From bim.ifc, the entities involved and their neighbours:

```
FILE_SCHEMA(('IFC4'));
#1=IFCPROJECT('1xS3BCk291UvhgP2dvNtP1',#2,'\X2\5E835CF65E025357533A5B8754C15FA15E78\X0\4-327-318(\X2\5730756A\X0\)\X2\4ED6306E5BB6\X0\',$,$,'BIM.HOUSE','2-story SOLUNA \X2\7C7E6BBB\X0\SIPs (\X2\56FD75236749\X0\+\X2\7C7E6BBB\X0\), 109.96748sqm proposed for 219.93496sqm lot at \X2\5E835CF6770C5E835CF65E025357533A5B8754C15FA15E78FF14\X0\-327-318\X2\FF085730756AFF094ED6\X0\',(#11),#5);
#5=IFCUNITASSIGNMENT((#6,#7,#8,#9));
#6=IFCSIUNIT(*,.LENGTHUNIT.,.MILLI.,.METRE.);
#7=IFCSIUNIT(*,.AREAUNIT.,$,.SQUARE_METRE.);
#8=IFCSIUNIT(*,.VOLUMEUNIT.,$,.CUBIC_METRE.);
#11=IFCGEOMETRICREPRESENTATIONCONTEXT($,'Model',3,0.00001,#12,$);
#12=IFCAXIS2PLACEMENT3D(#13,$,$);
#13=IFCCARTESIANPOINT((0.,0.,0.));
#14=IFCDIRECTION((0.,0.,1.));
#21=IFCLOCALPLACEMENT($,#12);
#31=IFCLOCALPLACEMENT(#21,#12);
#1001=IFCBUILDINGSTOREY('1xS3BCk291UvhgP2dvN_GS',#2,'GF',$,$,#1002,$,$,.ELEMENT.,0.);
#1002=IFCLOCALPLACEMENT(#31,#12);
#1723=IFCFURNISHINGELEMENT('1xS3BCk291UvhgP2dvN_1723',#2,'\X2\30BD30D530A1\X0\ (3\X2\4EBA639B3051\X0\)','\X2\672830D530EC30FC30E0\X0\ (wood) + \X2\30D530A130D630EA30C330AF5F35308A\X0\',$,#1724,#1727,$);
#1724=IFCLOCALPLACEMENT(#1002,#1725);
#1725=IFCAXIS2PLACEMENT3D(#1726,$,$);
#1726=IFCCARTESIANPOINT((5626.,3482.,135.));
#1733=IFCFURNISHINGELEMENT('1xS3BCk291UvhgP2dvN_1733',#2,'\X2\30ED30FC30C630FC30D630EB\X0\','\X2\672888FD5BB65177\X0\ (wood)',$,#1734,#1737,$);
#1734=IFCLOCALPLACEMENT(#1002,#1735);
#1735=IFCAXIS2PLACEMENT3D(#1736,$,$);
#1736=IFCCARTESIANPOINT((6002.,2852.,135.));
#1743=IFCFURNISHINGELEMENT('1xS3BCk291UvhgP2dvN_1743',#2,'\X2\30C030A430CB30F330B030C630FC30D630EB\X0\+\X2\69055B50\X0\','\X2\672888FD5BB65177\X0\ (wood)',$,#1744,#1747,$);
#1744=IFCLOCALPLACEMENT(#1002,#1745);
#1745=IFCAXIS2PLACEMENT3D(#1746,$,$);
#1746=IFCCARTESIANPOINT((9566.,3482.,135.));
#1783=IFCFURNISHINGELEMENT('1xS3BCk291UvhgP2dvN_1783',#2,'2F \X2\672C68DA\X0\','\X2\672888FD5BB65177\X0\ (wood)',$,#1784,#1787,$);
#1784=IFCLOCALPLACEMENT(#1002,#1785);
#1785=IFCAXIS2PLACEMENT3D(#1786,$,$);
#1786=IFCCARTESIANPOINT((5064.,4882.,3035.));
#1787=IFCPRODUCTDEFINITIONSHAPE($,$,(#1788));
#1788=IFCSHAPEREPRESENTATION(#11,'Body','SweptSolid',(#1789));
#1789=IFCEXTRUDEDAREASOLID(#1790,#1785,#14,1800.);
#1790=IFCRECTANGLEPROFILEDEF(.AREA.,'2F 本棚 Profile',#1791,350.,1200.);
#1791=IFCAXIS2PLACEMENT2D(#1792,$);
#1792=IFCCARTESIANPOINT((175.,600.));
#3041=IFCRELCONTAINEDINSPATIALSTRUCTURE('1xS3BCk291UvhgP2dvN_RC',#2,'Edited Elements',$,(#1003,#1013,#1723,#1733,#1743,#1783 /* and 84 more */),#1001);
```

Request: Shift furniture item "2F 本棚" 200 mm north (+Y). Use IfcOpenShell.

```python
import ifcopenshell
import ifcopenshell.api.geometry
import ifcopenshell.util.placement

model = ifcopenshell.open("bim.ifc")

item = model.by_guid("1xS3BCk291UvhgP2dvN_1783")
matrix = ifcopenshell.util.placement.get_local_placement(item.ObjectPlacement)
matrix[1, 3] += 200.0
ifcopenshell.api.geometry.edit_object_placement(model, product=item, matrix=matrix, is_si=False)

print(ifcopenshell.util.placement.get_local_placement(item.ObjectPlacement).round(3) + 0.0)

model.write("bim_v2.ifc")
```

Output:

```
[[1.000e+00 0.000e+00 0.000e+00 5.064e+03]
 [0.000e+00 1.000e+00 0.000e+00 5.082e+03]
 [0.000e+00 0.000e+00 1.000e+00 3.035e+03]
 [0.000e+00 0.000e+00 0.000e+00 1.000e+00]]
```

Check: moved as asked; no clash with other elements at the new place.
